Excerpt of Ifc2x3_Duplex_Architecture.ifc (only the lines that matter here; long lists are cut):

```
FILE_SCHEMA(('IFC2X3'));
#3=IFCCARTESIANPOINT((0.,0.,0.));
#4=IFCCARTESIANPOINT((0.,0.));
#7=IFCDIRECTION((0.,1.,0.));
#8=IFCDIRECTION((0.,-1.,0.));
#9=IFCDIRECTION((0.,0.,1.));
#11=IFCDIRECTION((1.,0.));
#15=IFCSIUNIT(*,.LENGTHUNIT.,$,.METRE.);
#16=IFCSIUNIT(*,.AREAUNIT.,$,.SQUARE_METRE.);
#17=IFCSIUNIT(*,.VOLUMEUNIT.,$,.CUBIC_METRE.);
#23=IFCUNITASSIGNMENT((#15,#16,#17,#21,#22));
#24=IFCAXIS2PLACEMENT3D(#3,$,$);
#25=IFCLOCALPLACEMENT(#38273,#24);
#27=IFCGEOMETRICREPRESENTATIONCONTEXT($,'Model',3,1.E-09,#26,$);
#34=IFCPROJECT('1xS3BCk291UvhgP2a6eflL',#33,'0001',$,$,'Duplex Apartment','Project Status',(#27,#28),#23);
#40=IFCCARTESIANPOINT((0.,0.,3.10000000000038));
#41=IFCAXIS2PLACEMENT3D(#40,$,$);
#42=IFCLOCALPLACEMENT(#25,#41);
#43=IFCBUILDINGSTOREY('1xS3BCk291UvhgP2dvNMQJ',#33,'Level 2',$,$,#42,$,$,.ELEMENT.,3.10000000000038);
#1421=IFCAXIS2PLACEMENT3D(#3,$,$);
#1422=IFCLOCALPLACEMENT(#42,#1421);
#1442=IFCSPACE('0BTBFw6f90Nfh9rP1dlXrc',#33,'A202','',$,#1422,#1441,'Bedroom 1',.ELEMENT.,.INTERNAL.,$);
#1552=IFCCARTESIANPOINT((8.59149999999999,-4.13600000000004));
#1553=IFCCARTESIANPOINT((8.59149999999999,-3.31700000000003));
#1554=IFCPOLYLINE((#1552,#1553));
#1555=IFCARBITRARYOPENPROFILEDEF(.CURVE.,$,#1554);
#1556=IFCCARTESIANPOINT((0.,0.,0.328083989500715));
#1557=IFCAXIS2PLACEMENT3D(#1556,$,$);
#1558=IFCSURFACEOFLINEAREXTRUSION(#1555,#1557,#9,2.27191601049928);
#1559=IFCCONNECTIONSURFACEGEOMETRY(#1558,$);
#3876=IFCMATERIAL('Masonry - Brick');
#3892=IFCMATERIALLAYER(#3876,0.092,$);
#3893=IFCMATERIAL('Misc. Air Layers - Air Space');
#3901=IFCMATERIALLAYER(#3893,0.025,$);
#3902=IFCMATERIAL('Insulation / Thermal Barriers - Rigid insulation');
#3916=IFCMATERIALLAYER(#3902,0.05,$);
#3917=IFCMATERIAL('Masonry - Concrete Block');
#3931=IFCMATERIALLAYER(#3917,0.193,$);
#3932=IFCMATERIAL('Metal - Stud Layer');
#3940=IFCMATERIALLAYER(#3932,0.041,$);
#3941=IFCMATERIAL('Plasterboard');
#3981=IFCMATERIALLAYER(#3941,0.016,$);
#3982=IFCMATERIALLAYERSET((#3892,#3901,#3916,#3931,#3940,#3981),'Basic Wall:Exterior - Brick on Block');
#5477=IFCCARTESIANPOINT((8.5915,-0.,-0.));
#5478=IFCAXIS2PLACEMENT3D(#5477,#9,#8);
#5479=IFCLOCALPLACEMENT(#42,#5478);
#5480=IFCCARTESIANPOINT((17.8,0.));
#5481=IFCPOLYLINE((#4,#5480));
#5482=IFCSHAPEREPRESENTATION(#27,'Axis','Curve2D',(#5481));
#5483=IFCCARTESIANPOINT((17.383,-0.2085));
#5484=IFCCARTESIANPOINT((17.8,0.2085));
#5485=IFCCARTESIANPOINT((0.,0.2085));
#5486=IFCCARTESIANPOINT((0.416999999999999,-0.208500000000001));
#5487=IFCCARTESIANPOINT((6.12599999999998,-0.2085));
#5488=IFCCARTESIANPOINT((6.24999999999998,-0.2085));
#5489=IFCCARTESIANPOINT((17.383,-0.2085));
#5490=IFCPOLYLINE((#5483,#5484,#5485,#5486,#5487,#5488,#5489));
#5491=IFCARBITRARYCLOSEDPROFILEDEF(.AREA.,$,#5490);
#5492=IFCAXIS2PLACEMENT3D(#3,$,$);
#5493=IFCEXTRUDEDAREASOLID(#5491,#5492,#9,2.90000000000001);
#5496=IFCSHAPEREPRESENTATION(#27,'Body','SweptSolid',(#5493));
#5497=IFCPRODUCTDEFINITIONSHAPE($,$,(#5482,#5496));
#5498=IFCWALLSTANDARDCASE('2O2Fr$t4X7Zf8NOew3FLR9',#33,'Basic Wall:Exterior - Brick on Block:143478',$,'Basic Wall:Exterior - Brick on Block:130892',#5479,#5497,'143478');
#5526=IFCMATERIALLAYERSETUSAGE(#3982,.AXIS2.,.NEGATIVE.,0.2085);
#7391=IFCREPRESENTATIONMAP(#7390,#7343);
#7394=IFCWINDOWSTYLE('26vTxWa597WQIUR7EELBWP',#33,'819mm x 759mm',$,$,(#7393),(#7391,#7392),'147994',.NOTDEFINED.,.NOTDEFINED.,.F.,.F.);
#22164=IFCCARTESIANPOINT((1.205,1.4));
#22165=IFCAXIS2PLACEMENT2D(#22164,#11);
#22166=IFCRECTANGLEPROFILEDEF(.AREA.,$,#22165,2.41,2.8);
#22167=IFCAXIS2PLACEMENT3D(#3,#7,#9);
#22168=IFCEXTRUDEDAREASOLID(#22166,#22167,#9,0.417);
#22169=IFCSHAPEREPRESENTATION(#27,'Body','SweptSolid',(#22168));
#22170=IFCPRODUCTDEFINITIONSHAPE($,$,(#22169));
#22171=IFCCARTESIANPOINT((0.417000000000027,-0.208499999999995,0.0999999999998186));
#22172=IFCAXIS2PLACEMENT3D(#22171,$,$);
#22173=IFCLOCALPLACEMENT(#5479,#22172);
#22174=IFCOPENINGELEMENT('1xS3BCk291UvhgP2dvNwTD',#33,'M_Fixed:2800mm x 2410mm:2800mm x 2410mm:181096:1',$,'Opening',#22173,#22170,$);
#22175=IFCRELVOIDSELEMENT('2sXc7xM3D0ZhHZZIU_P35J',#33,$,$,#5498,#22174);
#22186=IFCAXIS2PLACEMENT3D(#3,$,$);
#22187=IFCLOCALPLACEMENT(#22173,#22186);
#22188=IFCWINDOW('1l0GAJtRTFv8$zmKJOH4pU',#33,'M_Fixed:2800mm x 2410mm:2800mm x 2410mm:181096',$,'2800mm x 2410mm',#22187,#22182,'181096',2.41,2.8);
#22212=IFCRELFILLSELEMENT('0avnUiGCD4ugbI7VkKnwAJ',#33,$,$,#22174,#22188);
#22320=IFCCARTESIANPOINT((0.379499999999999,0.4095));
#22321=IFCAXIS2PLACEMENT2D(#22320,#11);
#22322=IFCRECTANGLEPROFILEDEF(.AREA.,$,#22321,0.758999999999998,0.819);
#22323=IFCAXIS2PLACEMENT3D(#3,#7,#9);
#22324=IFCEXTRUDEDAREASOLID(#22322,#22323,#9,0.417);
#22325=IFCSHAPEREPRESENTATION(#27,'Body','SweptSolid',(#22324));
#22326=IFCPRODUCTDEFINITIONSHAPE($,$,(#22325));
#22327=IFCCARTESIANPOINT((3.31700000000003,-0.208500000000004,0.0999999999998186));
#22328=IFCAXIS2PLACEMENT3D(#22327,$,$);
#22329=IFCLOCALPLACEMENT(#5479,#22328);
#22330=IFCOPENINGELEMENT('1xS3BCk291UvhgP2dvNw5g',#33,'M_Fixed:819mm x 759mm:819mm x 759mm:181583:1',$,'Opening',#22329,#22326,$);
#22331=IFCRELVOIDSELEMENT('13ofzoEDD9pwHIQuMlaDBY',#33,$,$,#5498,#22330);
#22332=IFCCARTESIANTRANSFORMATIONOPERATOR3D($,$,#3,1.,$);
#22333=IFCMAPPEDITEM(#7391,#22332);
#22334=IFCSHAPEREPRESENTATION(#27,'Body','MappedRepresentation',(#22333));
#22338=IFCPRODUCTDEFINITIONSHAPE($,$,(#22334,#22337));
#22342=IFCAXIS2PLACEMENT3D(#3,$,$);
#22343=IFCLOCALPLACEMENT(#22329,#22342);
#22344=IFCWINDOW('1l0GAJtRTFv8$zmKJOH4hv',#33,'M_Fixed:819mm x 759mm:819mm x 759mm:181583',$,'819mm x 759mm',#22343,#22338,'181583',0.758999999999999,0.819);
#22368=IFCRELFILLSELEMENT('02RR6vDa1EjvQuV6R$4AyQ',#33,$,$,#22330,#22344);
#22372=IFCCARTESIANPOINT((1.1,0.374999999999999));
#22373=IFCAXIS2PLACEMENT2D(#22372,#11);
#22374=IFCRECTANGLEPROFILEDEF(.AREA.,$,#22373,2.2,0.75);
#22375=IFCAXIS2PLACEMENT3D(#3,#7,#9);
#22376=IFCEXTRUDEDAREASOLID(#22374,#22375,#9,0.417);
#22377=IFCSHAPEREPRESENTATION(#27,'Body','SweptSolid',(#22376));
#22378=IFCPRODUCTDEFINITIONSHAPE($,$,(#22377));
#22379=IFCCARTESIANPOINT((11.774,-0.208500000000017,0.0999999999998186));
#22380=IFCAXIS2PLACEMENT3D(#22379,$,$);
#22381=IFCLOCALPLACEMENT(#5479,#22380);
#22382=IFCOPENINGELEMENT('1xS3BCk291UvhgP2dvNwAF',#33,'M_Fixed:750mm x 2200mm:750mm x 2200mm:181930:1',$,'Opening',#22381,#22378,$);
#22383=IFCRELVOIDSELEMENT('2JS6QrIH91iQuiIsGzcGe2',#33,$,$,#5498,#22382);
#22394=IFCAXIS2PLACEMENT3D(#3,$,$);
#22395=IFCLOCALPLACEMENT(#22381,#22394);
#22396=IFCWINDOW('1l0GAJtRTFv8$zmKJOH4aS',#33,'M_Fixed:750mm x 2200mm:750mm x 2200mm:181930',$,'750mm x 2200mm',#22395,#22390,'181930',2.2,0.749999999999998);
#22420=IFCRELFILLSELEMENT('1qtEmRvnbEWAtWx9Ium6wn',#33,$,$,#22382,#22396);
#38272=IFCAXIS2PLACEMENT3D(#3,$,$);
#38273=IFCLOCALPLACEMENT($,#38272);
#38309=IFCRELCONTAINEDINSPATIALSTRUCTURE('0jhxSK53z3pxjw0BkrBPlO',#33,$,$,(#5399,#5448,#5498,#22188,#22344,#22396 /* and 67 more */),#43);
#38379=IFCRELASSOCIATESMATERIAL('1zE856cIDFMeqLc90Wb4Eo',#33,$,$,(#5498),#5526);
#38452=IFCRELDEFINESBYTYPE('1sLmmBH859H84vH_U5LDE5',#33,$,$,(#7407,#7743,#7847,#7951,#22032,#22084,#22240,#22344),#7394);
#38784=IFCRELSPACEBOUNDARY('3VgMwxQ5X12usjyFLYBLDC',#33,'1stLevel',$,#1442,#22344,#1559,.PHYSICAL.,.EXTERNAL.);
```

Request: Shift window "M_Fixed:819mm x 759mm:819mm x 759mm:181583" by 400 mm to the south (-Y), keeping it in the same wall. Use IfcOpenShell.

```python
import numpy as np
import ifcopenshell
import ifcopenshell.api.geometry
import ifcopenshell.util.placement

model = ifcopenshell.open("Ifc2x3_Duplex_Architecture.ifc")

window = model.by_id(22344)
opening = window.FillsVoids[0].RelatingOpeningElement
wall = opening.VoidsElements[0].RelatingBuildingElement

wall_matrix = ifcopenshell.util.placement.get_local_placement(wall.ObjectPlacement)
shift = wall_matrix[:3, 0] * 0.4
before = ifcopenshell.util.placement.get_local_placement(window.ObjectPlacement)[:3, 3].copy()

# The window is placed relative to its opening, so it follows when the opening moves.
matrix = ifcopenshell.util.placement.get_local_placement(opening.ObjectPlacement)
matrix[:3, 3] += shift
ifcopenshell.api.geometry.edit_object_placement(
    model, product=opening, matrix=matrix, is_si=False, should_transform_children=True
)

# Space boundary surfaces are stored in each space's coordinates; move them too.
for rel in window.ProvidesBoundaries:
    if not rel.ConnectionGeometry:
        continue
    surface = rel.ConnectionGeometry.SurfaceOnRelatingElement
    space_matrix = ifcopenshell.util.placement.get_local_placement(rel.RelatingSpace.ObjectPlacement)
    point = np.array(surface.Position.Location.Coordinates) + space_matrix[:3, :3].T @ shift
    surface.Position = model.createIfcAxis2Placement3D(
        model.createIfcCartesianPoint(point.tolist()), surface.Position.Axis, surface.Position.RefDirection
    )

after = ifcopenshell.util.placement.get_local_placement(window.ObjectPlacement)[:3, 3]
print("window moved by", (after - before).round(3) + 0.0)

model.write("Ifc2x3_Duplex_Architecture_updated.ifc")
```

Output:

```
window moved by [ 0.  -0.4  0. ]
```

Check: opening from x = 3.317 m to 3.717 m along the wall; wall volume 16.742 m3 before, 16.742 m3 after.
